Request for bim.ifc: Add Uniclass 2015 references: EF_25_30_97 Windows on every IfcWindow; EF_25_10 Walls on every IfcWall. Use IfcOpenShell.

First a look at what the model holds.

```python
import ifcopenshell

model = ifcopenshell.open("bim.ifc")
print(model.schema)
print("classifications:", [c.Name for c in model.by_type("IfcClassification")])
for ifc_class in ("IfcDoor", "IfcRoof", "IfcStair", "IfcWall", "IfcWindow"):
    print(ifc_class, len(model.by_type(ifc_class)))
```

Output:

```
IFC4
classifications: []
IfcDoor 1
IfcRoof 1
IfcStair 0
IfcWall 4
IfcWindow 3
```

```python
import ifcopenshell
import ifcopenshell.api.classification

model = ifcopenshell.open("bim.ifc")

system = ifcopenshell.api.classification.add_classification(model, classification="Uniclass 2015")

codes = {
    "IfcWindow": ("EF_25_30_97", "Windows"),
    "IfcWall": ("EF_25_10", "Walls"),
}
for ifc_class, (code, name) in codes.items():
    products = model.by_type(ifc_class)
    ifcopenshell.api.classification.add_reference(
        model, products=products, classification=system, identification=code, name=name
    )
    print(code, len(products))

model.write("bim_v2.ifc")
```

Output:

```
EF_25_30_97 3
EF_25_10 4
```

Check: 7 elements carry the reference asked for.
